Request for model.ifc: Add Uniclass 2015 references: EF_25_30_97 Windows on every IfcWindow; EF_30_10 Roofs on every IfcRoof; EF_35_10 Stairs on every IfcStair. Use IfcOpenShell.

First a look at what the model holds.

```python
import ifcopenshell

model = ifcopenshell.open("model.ifc")
print(model.schema)
print("classifications:", [c.Name for c in model.by_type("IfcClassification")])
for ifc_class in ("IfcDoor", "IfcRoof", "IfcStair", "IfcWall", "IfcWindow"):
    print(ifc_class, len(model.by_type(ifc_class)))
```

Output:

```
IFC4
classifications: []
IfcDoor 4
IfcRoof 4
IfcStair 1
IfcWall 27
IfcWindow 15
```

```python
import ifcopenshell
import ifcopenshell.api.classification

model = ifcopenshell.open("model.ifc")

system = ifcopenshell.api.classification.add_classification(model, classification="Uniclass 2015")

codes = {
    "IfcWindow": ("EF_25_30_97", "Windows"),
    "IfcRoof": ("EF_30_10", "Roofs"),
    "IfcStair": ("EF_35_10", "Stairs"),
}
for ifc_class, (code, name) in codes.items():
    products = model.by_type(ifc_class)
    ifcopenshell.api.classification.add_reference(
        model, products=products, classification=system, identification=code, name=name
    )
    print(code, len(products))

model.write("model-out.ifc")
```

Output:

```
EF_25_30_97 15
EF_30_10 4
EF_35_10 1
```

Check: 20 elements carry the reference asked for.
